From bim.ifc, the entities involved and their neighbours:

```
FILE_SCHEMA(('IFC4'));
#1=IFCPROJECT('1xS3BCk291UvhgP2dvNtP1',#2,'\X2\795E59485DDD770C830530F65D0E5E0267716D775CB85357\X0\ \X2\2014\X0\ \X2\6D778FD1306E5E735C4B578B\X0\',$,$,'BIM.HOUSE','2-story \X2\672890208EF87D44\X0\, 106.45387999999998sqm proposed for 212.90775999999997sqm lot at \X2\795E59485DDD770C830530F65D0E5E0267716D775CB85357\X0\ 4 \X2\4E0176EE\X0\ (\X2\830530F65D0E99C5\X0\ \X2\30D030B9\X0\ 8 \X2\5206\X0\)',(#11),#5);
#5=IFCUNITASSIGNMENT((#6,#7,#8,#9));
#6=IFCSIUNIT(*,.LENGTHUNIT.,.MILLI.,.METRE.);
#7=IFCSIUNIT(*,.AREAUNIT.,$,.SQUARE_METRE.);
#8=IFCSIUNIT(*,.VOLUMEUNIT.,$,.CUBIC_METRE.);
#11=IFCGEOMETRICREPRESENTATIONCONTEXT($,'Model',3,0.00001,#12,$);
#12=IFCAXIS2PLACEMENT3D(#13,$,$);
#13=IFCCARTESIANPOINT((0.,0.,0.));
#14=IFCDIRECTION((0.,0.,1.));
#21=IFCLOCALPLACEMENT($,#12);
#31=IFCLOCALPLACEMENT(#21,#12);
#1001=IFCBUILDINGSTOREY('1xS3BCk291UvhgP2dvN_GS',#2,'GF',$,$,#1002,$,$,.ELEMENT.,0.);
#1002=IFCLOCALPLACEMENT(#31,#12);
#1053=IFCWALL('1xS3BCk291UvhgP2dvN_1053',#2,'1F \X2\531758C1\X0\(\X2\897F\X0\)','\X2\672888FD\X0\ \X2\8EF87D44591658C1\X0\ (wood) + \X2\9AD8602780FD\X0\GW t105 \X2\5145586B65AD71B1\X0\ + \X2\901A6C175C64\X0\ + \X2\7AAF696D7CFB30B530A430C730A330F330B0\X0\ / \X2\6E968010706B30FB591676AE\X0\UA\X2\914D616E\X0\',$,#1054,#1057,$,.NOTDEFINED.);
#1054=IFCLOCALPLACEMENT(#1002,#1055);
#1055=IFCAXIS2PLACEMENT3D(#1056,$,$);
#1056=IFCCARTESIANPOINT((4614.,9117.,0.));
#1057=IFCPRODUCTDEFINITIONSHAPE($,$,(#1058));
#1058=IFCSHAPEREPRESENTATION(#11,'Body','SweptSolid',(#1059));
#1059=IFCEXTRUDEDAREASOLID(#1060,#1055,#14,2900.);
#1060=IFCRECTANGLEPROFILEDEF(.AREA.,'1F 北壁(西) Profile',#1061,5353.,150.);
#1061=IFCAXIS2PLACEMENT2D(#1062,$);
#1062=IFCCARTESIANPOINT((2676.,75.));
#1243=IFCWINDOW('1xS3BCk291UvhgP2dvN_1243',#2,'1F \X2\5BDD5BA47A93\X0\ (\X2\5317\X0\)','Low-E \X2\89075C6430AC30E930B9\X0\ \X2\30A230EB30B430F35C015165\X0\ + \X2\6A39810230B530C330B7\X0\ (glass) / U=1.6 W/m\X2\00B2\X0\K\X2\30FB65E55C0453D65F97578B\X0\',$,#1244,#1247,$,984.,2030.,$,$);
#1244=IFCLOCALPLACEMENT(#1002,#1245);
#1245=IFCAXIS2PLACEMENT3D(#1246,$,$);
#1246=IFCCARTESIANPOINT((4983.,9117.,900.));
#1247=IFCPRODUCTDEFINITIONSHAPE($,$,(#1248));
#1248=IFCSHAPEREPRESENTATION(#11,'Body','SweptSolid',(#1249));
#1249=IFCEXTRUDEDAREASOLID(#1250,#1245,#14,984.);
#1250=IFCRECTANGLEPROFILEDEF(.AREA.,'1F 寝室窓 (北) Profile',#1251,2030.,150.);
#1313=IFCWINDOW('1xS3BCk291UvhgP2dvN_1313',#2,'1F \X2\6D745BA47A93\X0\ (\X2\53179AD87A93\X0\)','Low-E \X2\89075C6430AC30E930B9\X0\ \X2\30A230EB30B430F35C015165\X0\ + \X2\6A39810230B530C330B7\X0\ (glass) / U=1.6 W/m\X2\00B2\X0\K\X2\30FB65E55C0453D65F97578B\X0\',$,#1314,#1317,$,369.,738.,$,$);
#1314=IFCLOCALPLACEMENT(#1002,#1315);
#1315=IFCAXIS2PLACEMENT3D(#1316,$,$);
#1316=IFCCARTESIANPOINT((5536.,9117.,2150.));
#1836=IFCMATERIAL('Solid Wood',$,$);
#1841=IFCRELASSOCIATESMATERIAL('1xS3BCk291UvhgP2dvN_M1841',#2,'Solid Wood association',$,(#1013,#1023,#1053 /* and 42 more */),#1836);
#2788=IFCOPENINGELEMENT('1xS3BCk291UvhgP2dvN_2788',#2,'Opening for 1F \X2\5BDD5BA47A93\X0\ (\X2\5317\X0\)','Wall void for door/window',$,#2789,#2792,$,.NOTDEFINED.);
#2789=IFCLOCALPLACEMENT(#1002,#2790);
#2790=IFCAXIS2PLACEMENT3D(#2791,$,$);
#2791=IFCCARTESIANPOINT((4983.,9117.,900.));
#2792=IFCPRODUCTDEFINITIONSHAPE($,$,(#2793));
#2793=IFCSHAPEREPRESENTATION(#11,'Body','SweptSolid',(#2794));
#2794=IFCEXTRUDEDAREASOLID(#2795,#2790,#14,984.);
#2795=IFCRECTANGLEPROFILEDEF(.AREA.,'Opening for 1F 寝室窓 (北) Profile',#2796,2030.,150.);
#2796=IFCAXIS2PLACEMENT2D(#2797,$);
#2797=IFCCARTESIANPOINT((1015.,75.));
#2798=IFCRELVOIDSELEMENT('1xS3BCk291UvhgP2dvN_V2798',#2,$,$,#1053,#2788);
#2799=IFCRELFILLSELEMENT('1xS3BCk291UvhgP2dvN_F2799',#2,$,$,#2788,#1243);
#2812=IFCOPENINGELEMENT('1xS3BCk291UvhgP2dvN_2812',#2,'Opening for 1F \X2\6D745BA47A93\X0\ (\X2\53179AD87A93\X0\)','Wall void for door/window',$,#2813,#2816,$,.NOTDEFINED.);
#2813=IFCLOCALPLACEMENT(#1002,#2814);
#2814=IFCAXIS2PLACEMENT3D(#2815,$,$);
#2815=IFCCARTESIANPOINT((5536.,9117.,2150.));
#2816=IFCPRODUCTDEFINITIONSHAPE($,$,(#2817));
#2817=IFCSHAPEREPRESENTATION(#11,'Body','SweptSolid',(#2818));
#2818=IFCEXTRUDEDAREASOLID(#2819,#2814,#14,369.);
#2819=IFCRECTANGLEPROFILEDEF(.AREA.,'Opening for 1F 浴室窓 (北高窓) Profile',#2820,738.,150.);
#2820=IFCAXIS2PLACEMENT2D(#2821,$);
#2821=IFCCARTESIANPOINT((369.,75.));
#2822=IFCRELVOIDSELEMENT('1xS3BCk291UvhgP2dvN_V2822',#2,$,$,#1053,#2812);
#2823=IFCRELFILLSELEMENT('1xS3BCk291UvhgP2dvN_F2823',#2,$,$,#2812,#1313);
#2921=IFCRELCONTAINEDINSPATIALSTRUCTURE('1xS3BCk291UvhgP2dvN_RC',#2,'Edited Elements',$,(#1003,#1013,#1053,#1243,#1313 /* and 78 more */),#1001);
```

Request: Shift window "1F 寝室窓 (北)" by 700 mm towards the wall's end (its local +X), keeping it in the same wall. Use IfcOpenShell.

```python
import ifcopenshell
import ifcopenshell.api.geometry
import ifcopenshell.util.placement
import ifcopenshell.util.unit

model = ifcopenshell.open("bim.ifc")
unit_scale = ifcopenshell.util.unit.calculate_unit_scale(model)

window = model.by_guid("1xS3BCk291UvhgP2dvN_1243")
opening = window.FillsVoids[0].RelatingOpeningElement
wall = opening.VoidsElements[0].RelatingBuildingElement

wall_matrix = ifcopenshell.util.placement.get_local_placement(wall.ObjectPlacement)
shift = wall_matrix[:3, 0] * 0.7 / unit_scale
before = ifcopenshell.util.placement.get_local_placement(window.ObjectPlacement)[:3, 3].copy()

# The window is not placed relative to its opening, so move both.
for product in (opening, window):
    matrix = ifcopenshell.util.placement.get_local_placement(product.ObjectPlacement)
    matrix[:3, 3] += shift
    ifcopenshell.api.geometry.edit_object_placement(model, product=product, matrix=matrix, is_si=False)

after = ifcopenshell.util.placement.get_local_placement(window.ObjectPlacement)[:3, 3]
print("window moved by", (after - before).round(3) + 0.0)

model.write("bim_updated.ifc")
```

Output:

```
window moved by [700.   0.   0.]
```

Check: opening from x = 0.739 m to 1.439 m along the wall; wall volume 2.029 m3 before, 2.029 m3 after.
